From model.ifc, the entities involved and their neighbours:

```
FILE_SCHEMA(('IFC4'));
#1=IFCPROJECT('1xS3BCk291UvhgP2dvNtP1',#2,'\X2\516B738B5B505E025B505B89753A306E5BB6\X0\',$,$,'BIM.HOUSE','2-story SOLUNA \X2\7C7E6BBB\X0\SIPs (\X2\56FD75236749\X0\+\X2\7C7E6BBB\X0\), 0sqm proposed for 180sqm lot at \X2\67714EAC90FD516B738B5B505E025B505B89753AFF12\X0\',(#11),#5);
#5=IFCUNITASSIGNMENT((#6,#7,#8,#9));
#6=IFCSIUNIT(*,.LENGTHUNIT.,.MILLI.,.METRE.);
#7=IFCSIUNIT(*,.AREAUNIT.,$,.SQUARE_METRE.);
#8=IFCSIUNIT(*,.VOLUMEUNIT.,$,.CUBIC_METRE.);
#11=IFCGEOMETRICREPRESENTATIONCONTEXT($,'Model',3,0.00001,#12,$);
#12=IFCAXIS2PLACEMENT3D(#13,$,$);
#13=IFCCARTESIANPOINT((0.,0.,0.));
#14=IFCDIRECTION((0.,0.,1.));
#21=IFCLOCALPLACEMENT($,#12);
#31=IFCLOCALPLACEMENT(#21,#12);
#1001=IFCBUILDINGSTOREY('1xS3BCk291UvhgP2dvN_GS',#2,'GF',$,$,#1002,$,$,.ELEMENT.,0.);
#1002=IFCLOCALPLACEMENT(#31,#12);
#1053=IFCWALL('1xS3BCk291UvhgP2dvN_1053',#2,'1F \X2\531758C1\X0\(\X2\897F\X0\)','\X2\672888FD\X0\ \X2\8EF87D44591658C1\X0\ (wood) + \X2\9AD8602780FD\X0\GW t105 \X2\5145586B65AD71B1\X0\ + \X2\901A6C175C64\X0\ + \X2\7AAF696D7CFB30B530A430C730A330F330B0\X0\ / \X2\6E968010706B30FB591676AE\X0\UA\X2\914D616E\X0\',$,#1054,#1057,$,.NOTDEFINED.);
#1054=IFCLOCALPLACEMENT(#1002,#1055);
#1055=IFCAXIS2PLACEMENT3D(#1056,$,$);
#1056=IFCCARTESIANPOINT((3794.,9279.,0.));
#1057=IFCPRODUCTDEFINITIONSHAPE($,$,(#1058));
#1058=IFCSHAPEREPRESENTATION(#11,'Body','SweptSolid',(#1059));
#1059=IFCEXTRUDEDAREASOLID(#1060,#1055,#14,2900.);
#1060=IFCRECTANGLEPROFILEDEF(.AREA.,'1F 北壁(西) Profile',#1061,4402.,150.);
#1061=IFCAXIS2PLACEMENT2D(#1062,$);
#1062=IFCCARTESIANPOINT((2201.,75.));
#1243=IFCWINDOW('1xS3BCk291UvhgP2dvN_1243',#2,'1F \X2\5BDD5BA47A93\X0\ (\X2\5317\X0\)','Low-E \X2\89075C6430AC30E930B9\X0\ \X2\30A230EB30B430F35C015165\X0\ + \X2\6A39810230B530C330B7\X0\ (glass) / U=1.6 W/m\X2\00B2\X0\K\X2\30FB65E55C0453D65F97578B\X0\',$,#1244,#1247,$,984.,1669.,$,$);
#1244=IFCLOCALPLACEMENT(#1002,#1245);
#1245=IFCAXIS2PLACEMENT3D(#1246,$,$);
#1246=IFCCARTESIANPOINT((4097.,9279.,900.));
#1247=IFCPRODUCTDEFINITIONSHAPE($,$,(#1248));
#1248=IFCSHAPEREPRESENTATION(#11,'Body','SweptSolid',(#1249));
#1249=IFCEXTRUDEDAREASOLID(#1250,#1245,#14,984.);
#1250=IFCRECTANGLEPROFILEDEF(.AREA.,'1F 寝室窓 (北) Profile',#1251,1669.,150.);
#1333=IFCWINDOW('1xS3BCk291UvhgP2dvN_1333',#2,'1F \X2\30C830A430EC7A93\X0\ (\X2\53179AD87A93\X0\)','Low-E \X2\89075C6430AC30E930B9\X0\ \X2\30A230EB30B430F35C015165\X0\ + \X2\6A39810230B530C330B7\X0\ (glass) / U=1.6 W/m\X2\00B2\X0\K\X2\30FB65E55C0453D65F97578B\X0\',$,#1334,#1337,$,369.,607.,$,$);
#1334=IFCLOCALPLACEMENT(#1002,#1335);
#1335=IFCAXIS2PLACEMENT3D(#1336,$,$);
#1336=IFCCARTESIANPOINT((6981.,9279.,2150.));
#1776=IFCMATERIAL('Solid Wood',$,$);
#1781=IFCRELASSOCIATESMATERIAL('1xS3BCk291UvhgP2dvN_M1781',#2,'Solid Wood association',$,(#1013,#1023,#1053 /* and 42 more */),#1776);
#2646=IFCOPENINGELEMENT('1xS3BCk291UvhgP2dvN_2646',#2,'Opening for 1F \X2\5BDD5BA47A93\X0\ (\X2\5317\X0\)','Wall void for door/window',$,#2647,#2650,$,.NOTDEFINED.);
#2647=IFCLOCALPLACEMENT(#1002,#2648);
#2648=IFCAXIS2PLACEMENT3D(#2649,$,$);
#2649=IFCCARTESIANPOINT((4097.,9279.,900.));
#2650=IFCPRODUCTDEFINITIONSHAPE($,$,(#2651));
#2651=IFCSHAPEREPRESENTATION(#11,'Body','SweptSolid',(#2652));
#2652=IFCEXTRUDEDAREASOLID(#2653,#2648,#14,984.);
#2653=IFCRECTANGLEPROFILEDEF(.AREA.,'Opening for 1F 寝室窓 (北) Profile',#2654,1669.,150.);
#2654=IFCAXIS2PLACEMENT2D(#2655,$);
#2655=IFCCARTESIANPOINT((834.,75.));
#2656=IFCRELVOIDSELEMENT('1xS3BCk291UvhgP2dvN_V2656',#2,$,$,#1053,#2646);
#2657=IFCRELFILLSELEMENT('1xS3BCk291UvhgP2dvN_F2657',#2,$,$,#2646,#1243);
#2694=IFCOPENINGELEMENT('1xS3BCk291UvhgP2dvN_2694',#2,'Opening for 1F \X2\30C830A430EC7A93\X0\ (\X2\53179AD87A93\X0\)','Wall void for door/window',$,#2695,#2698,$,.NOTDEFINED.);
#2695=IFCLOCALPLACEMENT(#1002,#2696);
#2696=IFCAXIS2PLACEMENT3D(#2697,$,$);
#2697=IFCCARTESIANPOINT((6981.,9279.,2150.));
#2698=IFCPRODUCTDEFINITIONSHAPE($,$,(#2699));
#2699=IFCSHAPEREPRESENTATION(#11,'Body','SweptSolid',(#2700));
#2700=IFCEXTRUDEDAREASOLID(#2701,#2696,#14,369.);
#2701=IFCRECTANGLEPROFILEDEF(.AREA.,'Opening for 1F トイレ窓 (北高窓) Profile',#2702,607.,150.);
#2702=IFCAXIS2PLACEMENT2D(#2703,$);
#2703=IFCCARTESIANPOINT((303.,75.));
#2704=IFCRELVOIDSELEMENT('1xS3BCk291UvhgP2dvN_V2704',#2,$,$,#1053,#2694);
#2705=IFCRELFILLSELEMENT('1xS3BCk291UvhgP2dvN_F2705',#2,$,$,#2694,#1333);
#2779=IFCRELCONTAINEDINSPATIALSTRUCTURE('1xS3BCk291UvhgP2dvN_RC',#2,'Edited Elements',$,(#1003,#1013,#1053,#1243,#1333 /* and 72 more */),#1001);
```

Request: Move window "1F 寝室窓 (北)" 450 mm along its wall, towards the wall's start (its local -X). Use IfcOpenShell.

```python
import ifcopenshell
import ifcopenshell.api.geometry
import ifcopenshell.util.placement
import ifcopenshell.util.unit

model = ifcopenshell.open("model.ifc")
unit_scale = ifcopenshell.util.unit.calculate_unit_scale(model)

window = model.by_guid("1xS3BCk291UvhgP2dvN_1243")
opening = window.FillsVoids[0].RelatingOpeningElement
wall = opening.VoidsElements[0].RelatingBuildingElement

wall_matrix = ifcopenshell.util.placement.get_local_placement(wall.ObjectPlacement)
shift = wall_matrix[:3, 0] * -0.45 / unit_scale
before = ifcopenshell.util.placement.get_local_placement(window.ObjectPlacement)[:3, 3].copy()

# The window is not placed relative to its opening, so move both.
for product in (opening, window):
    matrix = ifcopenshell.util.placement.get_local_placement(product.ObjectPlacement)
    matrix[:3, 3] += shift
    ifcopenshell.api.geometry.edit_object_placement(model, product=product, matrix=matrix, is_si=False)

after = ifcopenshell.util.placement.get_local_placement(window.ObjectPlacement)[:3, 3]
print("window moved by", (after - before).round(3) + 0.0)

model.write("model_edited.ifc")
```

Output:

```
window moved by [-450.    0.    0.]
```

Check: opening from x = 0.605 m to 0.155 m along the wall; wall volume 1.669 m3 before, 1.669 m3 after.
